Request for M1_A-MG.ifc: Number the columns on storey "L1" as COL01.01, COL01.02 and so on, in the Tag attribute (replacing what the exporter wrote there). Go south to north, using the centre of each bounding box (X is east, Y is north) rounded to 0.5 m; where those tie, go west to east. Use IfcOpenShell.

First a look at what the model holds.

```python
import ifcopenshell
import ifcopenshell.util.element
import ifcopenshell.util.placement

model = ifcopenshell.open("M1_A-MG.ifc")
print(model.schema)
storey = next(s for s in model.by_type("IfcBuildingStorey") if s.Name == "L1")
columns = [e for e in ifcopenshell.util.element.get_decomposition(storey) if e.is_a("IfcColumn")]
for e in sorted(columns, key=lambda e: e.id()):
    origin = ifcopenshell.util.placement.get_local_placement(e.ObjectPlacement)[:3, 3]
    print(e.id(), e.Tag, e.Name, origin.round(2) + 0.0, sep=" | ")
```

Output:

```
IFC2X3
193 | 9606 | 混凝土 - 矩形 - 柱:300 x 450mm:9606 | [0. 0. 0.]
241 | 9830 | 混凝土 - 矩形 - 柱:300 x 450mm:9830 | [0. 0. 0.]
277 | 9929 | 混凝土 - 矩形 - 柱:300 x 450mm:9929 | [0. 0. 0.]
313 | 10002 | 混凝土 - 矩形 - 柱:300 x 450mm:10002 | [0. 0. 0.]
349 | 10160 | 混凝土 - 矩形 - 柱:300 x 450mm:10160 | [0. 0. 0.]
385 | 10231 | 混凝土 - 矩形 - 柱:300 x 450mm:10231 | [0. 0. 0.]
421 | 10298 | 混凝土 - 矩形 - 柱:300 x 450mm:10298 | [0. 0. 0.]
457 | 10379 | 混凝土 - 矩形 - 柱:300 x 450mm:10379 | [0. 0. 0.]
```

```python
import ifcopenshell
import ifcopenshell.geom
import ifcopenshell.util.element
import ifcopenshell.util.shape

model = ifcopenshell.open("M1_A-MG.ifc")
settings = ifcopenshell.geom.settings()
settings.set("use-world-coords", True)


def centre(element):
    shape = ifcopenshell.geom.create_shape(settings, element)
    return ifcopenshell.util.shape.get_bbox_centroid(shape.geometry)


storey = next(s for s in model.by_type("IfcBuildingStorey") if s.Name == "L1")
columns = [e for e in ifcopenshell.util.element.get_decomposition(storey) if e.is_a("IfcColumn")]

# Insertion points can sit at a corner or the storey origin, so sort by the geometry (in metres).
centres = {e: centre(e) for e in columns}
columns.sort(key=lambda e: (round(centres[e][1] / 0.5), centres[e][0]))

for i, e in enumerate(columns, start=1):
    number = f"COL01.{i:02d}"
    e.Tag = number
    print(e.id(), number)

model.write("M1_A-MG-out.ifc")
```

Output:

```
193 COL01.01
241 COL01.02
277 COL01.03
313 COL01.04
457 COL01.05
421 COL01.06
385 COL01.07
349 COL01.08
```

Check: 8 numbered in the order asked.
